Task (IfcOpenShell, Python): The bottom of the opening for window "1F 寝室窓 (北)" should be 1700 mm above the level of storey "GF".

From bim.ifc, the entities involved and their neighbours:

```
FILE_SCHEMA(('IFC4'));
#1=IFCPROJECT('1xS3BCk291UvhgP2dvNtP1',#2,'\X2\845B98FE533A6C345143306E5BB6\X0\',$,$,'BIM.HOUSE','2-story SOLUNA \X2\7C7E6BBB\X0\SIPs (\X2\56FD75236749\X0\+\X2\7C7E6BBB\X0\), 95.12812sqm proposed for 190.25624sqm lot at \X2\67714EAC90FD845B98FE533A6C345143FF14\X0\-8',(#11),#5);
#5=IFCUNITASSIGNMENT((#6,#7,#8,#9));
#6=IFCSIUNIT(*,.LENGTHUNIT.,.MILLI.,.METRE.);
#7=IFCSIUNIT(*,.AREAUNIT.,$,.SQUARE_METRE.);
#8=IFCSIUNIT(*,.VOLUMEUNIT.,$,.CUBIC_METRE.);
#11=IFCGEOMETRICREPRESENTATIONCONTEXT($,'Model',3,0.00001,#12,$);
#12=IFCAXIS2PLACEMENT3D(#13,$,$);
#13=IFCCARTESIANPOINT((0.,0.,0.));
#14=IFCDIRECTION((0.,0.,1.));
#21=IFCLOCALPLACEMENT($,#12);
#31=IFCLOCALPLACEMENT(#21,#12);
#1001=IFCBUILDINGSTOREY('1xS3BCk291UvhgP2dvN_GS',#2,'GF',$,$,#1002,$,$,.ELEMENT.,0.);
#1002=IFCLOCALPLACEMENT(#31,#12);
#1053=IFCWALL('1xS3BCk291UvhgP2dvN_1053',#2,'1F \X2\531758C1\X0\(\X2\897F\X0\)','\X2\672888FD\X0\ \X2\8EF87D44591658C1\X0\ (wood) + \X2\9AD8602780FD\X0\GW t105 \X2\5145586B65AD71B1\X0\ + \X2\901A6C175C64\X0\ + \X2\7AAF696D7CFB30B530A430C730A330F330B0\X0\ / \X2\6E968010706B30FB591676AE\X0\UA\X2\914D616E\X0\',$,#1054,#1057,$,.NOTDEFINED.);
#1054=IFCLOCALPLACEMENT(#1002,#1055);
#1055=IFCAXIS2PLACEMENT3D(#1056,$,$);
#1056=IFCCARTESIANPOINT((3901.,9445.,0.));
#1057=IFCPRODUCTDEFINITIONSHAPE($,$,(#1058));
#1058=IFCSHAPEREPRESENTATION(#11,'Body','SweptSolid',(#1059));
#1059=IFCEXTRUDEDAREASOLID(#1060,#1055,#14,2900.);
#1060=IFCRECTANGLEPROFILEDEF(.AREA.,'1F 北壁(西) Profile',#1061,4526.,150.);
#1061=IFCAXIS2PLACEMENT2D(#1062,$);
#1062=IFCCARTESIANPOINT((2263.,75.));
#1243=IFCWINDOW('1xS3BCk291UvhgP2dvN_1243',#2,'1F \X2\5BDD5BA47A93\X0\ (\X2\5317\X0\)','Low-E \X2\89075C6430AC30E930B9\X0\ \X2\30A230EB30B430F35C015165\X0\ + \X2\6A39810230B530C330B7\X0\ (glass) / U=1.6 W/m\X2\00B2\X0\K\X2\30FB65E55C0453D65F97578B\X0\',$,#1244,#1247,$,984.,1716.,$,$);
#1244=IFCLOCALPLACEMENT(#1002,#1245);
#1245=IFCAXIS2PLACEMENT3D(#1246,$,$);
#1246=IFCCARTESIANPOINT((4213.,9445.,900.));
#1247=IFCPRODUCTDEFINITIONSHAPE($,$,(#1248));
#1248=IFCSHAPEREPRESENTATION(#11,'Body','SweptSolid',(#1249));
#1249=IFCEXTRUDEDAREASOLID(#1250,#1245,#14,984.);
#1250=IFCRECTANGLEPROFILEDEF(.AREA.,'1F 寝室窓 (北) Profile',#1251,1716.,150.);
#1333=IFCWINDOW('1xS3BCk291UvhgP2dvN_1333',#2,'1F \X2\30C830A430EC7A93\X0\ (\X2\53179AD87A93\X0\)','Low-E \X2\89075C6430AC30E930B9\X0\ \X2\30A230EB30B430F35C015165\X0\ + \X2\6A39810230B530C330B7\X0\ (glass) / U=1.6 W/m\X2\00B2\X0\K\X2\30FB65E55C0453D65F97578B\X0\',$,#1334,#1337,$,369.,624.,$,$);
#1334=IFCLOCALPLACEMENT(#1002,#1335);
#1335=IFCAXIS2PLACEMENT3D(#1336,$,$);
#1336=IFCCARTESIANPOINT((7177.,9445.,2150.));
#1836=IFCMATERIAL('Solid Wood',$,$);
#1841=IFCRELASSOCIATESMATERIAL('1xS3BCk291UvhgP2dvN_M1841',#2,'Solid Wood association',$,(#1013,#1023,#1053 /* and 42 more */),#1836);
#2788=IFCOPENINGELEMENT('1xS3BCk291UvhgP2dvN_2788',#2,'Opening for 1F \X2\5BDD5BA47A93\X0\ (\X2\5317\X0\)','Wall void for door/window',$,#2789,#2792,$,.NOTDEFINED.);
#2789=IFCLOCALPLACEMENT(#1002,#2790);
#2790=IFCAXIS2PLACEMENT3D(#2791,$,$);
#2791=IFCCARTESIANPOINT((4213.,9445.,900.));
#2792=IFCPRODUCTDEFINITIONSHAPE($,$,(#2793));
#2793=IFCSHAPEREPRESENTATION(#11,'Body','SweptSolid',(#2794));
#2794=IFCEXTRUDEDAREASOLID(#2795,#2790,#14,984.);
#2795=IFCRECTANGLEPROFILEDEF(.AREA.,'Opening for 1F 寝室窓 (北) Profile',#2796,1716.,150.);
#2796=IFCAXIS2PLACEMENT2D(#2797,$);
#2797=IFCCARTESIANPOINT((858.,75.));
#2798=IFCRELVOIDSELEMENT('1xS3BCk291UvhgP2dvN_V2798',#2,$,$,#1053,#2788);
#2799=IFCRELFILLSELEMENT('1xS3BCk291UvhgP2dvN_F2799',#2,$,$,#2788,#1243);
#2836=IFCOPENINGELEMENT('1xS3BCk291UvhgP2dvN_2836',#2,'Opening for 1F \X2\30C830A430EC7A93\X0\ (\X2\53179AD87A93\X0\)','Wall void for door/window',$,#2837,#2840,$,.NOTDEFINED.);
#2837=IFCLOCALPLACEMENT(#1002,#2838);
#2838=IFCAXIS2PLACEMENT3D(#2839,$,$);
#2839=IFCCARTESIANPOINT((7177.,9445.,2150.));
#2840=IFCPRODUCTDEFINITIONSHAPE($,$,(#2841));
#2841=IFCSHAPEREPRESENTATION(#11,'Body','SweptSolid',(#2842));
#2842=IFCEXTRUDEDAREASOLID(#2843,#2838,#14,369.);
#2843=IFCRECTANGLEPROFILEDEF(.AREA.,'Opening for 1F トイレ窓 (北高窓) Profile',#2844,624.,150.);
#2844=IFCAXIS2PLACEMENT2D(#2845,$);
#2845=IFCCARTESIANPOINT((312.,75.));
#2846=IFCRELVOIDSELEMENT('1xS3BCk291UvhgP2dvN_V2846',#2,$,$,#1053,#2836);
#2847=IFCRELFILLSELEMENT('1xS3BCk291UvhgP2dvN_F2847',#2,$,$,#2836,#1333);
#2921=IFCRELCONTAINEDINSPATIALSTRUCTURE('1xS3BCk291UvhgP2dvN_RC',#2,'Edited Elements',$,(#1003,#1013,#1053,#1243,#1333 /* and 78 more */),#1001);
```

```python
import numpy as np
import ifcopenshell
import ifcopenshell.api.geometry
import ifcopenshell.geom
import ifcopenshell.util.element
import ifcopenshell.util.placement
import ifcopenshell.util.shape
import ifcopenshell.util.unit

model = ifcopenshell.open("bim.ifc")
unit_scale = ifcopenshell.util.unit.calculate_unit_scale(model)

window = model.by_guid("1xS3BCk291UvhgP2dvN_1243")
opening = window.FillsVoids[0].RelatingOpeningElement
storey = ifcopenshell.util.element.get_container(window, ifc_class="IfcBuildingStorey")
level = ifcopenshell.util.placement.get_local_placement(storey.ObjectPlacement)[2, 3]

# The opening's origin need not be at the sill, so measure its lowest point.
shape = ifcopenshell.geom.create_shape(ifcopenshell.geom.settings(), opening)
bottom = ifcopenshell.util.shape.get_shape_bottom_elevation(shape, shape.geometry) / unit_scale
dz = level + 1.7 / unit_scale - bottom

shift = np.array([0.0, 0.0, dz])
# The window is not placed relative to its opening, so move both.
for product in (opening, window):
    matrix = ifcopenshell.util.placement.get_local_placement(product.ObjectPlacement)
    matrix[:3, 3] += shift
    ifcopenshell.api.geometry.edit_object_placement(model, product=product, matrix=matrix, is_si=False)

print(f"moved by {dz * unit_scale:+.3f} m")

model.write("bim_updated.ifc")
```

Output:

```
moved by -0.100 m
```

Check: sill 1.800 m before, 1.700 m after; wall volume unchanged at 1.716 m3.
